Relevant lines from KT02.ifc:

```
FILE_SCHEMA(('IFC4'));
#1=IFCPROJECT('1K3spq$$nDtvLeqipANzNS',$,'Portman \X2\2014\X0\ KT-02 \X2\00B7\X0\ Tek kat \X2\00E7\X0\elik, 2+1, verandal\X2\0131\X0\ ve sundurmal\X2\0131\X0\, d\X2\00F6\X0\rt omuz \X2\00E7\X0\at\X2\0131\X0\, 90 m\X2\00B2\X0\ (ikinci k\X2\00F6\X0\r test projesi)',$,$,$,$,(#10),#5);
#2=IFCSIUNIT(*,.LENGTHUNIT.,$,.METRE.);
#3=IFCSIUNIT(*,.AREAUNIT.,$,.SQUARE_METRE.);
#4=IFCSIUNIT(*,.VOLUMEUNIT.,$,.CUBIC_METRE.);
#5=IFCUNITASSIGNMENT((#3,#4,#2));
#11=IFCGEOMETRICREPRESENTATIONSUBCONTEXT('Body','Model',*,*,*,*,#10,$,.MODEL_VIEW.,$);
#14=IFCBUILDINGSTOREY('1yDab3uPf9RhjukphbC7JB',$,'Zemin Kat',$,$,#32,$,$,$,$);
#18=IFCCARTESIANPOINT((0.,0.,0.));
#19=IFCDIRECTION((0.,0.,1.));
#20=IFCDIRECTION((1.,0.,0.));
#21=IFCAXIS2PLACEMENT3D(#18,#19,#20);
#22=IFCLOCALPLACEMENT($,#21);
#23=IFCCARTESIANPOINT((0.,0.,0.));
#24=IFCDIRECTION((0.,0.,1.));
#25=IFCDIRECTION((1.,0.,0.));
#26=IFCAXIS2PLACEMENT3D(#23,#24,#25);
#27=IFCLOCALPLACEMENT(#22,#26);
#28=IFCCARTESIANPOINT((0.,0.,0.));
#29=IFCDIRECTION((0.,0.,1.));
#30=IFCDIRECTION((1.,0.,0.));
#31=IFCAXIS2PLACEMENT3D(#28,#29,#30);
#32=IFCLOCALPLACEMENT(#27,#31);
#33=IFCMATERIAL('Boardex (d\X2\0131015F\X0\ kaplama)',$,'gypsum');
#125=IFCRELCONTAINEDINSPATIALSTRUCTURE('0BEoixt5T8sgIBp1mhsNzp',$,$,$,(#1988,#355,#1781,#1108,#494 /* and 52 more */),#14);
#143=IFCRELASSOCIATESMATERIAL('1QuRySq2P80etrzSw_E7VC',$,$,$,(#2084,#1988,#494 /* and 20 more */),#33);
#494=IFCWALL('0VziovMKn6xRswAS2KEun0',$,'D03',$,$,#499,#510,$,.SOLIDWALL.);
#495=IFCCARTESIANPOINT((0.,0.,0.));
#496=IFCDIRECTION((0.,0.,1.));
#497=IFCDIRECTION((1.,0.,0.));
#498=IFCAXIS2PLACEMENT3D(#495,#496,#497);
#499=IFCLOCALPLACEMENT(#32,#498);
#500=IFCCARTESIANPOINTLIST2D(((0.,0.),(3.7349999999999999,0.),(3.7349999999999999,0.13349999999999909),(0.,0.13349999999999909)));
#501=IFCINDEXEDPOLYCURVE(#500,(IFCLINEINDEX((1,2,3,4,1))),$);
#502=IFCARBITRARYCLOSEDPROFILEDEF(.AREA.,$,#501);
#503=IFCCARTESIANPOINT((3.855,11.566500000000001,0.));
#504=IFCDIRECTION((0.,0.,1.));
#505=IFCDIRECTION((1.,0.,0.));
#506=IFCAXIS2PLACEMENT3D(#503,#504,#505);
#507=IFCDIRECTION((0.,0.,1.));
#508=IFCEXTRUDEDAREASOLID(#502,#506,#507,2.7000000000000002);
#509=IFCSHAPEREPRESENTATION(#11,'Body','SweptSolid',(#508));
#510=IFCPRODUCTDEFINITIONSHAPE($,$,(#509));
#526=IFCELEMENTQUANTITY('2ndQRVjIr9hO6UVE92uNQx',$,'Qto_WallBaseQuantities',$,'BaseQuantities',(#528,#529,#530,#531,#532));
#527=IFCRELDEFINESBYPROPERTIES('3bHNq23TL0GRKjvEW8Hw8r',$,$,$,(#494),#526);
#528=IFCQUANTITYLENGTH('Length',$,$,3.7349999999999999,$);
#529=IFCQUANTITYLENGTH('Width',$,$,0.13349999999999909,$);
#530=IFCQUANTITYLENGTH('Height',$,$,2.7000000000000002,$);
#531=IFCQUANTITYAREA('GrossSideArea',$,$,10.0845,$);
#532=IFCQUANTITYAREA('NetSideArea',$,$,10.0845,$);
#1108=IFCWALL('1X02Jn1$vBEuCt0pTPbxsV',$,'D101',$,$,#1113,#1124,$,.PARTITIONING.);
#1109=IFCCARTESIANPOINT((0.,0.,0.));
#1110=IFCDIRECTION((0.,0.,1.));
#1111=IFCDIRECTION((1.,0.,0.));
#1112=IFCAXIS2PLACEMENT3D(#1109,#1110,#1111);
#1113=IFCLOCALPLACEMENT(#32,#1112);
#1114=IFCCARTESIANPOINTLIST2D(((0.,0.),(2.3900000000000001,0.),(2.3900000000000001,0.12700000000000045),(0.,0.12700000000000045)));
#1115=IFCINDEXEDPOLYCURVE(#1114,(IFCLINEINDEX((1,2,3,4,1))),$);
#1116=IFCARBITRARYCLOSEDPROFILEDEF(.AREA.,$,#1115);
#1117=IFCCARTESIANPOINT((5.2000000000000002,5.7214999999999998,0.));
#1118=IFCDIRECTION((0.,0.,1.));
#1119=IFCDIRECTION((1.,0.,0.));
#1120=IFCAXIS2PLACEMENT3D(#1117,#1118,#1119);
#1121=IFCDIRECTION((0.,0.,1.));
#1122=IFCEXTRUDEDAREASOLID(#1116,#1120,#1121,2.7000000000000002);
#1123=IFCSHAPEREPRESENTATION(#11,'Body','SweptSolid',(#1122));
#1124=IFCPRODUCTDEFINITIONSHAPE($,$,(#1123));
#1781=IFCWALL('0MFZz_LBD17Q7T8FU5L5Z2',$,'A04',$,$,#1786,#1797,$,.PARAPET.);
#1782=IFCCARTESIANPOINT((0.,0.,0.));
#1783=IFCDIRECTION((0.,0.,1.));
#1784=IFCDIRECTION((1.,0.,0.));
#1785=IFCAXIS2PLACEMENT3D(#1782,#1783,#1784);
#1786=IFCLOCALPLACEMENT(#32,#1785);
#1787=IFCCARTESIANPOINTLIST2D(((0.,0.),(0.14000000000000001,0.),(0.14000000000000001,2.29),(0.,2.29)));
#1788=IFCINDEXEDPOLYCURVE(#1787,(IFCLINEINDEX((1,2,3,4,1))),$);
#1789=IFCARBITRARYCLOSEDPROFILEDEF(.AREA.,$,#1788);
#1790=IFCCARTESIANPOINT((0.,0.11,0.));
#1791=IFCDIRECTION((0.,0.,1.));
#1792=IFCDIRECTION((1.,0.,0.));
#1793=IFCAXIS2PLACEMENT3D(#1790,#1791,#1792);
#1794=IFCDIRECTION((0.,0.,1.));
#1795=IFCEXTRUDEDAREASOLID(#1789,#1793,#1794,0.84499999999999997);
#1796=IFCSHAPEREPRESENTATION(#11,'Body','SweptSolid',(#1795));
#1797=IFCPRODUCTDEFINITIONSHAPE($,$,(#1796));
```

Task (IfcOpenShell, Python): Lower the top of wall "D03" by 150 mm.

```python
import ifcopenshell
import ifcopenshell.api.pset
import ifcopenshell.geom
import ifcopenshell.util.element
import ifcopenshell.util.representation
import ifcopenshell.util.shape
import ifcopenshell.util.unit

model = ifcopenshell.open("KT02.ifc")
unit_scale = ifcopenshell.util.unit.calculate_unit_scale(model)
area_scale = ifcopenshell.util.unit.calculate_unit_scale(model, "AREAUNIT")
settings = ifcopenshell.geom.settings()


def volume(element):
    """Net volume in cubic metres, openings subtracted."""
    shape = ifcopenshell.geom.create_shape(settings, element)
    return ifcopenshell.util.shape.get_volume(shape.geometry)


wall = model.by_guid("0VziovMKn6xRswAS2KEun0")
before = volume(wall)

body = ifcopenshell.util.representation.get_representation(wall, "Model", "Body")
solid = body.Items[0]
old_height = solid.Depth
solid.Depth -= 0.15 / unit_scale
after = volume(wall)
thickness = 0.1335  # wall thickness in metres

# Update the stored height, areas and volumes.
qto = model.by_id(ifcopenshell.util.element.get_pset(wall, "Qto_WallBaseQuantities", should_inherit=False)["id"])
ifcopenshell.api.pset.edit_qto(model, qto=qto, properties={
    "Height": solid.Depth,
    "GrossSideArea": ifcopenshell.util.element.get_pset(wall, "Qto_WallBaseQuantities", "GrossSideArea") * solid.Depth / old_height,
    "NetSideArea": after / thickness / area_scale,
})

print(f"height {old_height:g} -> {solid.Depth:g}, volume {before:.3f} -> {after:.3f} m3")

model.write("KT02_updated.ifc")
```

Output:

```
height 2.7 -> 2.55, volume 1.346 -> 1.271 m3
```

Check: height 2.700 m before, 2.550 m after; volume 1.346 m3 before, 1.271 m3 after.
